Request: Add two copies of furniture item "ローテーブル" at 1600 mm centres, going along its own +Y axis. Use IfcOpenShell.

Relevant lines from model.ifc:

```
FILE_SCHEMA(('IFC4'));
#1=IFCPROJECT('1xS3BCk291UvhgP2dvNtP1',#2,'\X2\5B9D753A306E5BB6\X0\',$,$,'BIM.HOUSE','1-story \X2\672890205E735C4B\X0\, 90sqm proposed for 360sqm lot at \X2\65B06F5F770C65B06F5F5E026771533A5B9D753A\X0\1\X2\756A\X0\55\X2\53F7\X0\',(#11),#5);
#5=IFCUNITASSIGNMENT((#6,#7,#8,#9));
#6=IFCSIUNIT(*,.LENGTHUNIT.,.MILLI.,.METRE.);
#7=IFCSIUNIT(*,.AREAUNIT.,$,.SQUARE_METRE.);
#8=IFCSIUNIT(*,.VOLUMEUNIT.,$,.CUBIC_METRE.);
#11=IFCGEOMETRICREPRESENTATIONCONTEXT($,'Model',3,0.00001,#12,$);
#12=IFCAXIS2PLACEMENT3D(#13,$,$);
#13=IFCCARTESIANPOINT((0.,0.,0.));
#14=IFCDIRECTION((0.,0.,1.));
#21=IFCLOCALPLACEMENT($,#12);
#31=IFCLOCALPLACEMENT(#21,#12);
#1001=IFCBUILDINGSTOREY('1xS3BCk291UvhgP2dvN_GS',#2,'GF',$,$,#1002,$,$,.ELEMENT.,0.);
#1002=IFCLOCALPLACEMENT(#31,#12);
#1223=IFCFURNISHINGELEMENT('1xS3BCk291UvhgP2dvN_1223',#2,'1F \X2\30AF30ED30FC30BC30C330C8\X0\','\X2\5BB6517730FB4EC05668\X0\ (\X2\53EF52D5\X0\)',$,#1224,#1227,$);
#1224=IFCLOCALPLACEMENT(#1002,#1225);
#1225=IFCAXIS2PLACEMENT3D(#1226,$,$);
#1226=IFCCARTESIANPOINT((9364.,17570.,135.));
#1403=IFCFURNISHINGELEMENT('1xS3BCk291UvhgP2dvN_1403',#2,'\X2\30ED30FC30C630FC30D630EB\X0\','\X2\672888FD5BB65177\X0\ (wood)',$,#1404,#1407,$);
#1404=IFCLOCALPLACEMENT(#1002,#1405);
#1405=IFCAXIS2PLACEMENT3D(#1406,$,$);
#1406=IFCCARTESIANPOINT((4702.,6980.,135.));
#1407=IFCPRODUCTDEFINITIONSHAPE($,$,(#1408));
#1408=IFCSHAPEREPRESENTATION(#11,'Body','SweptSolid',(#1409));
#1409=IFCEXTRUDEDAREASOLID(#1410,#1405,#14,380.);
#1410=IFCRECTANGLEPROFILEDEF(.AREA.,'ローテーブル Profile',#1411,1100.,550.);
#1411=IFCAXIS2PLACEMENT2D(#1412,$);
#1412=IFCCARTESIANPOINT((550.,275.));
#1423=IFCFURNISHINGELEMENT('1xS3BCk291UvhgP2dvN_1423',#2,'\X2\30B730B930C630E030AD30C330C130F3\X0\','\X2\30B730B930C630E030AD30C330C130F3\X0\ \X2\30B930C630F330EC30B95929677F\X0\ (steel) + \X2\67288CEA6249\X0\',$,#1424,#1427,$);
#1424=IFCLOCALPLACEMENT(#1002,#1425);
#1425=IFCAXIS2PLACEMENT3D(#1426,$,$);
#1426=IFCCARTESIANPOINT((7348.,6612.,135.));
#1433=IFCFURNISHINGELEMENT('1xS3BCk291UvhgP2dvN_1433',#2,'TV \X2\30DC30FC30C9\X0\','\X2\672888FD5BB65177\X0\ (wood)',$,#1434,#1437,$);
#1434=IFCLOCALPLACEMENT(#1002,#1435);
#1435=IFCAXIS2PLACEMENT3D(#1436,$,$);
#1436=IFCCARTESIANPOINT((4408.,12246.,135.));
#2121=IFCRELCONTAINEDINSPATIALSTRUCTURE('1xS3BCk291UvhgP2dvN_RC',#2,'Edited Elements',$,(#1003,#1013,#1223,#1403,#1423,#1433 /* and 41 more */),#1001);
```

```python
import ifcopenshell
import ifcopenshell.api.geometry
import ifcopenshell.api.root
import ifcopenshell.util.element
import ifcopenshell.util.placement
import ifcopenshell.util.unit

model = ifcopenshell.open("model.ifc")
unit_scale = ifcopenshell.util.unit.calculate_unit_scale(model)


def reuse_history(source, copy):
    """copy_class also copies each property set's owner history, people and application; keep the originals."""
    for rel in copy.IsDefinedBy:
        if rel.is_a("IfcRelDefinesByProperties") and (history := rel.RelatingPropertyDefinition.OwnerHistory):
            rel.RelatingPropertyDefinition.OwnerHistory = source.OwnerHistory
            ifcopenshell.util.element.remove_deep2(model, history)


source = model.by_guid("1xS3BCk291UvhgP2dvN_1403")
base = ifcopenshell.util.placement.get_local_placement(source.ObjectPlacement)
step = base[:3, 1] * 1.6 / unit_scale

for i in range(1, 3):
    copy = ifcopenshell.api.root.copy_class(model, product=source)
    copy.Representation = ifcopenshell.util.element.copy_deep(
        model, source.Representation, exclude=["IfcGeometricRepresentationContext", "IfcRepresentationMap"]
    )
    reuse_history(source, copy)
    matrix = base.copy()
    matrix[:3, 3] += i * step
    print("added at", matrix[:3, 3].round(3) + 0.0)
    ifcopenshell.api.geometry.edit_object_placement(model, product=copy, matrix=matrix, is_si=False)

model.write("model_v2.ifc")
```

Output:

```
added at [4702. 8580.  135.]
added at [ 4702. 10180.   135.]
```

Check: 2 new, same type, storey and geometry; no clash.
